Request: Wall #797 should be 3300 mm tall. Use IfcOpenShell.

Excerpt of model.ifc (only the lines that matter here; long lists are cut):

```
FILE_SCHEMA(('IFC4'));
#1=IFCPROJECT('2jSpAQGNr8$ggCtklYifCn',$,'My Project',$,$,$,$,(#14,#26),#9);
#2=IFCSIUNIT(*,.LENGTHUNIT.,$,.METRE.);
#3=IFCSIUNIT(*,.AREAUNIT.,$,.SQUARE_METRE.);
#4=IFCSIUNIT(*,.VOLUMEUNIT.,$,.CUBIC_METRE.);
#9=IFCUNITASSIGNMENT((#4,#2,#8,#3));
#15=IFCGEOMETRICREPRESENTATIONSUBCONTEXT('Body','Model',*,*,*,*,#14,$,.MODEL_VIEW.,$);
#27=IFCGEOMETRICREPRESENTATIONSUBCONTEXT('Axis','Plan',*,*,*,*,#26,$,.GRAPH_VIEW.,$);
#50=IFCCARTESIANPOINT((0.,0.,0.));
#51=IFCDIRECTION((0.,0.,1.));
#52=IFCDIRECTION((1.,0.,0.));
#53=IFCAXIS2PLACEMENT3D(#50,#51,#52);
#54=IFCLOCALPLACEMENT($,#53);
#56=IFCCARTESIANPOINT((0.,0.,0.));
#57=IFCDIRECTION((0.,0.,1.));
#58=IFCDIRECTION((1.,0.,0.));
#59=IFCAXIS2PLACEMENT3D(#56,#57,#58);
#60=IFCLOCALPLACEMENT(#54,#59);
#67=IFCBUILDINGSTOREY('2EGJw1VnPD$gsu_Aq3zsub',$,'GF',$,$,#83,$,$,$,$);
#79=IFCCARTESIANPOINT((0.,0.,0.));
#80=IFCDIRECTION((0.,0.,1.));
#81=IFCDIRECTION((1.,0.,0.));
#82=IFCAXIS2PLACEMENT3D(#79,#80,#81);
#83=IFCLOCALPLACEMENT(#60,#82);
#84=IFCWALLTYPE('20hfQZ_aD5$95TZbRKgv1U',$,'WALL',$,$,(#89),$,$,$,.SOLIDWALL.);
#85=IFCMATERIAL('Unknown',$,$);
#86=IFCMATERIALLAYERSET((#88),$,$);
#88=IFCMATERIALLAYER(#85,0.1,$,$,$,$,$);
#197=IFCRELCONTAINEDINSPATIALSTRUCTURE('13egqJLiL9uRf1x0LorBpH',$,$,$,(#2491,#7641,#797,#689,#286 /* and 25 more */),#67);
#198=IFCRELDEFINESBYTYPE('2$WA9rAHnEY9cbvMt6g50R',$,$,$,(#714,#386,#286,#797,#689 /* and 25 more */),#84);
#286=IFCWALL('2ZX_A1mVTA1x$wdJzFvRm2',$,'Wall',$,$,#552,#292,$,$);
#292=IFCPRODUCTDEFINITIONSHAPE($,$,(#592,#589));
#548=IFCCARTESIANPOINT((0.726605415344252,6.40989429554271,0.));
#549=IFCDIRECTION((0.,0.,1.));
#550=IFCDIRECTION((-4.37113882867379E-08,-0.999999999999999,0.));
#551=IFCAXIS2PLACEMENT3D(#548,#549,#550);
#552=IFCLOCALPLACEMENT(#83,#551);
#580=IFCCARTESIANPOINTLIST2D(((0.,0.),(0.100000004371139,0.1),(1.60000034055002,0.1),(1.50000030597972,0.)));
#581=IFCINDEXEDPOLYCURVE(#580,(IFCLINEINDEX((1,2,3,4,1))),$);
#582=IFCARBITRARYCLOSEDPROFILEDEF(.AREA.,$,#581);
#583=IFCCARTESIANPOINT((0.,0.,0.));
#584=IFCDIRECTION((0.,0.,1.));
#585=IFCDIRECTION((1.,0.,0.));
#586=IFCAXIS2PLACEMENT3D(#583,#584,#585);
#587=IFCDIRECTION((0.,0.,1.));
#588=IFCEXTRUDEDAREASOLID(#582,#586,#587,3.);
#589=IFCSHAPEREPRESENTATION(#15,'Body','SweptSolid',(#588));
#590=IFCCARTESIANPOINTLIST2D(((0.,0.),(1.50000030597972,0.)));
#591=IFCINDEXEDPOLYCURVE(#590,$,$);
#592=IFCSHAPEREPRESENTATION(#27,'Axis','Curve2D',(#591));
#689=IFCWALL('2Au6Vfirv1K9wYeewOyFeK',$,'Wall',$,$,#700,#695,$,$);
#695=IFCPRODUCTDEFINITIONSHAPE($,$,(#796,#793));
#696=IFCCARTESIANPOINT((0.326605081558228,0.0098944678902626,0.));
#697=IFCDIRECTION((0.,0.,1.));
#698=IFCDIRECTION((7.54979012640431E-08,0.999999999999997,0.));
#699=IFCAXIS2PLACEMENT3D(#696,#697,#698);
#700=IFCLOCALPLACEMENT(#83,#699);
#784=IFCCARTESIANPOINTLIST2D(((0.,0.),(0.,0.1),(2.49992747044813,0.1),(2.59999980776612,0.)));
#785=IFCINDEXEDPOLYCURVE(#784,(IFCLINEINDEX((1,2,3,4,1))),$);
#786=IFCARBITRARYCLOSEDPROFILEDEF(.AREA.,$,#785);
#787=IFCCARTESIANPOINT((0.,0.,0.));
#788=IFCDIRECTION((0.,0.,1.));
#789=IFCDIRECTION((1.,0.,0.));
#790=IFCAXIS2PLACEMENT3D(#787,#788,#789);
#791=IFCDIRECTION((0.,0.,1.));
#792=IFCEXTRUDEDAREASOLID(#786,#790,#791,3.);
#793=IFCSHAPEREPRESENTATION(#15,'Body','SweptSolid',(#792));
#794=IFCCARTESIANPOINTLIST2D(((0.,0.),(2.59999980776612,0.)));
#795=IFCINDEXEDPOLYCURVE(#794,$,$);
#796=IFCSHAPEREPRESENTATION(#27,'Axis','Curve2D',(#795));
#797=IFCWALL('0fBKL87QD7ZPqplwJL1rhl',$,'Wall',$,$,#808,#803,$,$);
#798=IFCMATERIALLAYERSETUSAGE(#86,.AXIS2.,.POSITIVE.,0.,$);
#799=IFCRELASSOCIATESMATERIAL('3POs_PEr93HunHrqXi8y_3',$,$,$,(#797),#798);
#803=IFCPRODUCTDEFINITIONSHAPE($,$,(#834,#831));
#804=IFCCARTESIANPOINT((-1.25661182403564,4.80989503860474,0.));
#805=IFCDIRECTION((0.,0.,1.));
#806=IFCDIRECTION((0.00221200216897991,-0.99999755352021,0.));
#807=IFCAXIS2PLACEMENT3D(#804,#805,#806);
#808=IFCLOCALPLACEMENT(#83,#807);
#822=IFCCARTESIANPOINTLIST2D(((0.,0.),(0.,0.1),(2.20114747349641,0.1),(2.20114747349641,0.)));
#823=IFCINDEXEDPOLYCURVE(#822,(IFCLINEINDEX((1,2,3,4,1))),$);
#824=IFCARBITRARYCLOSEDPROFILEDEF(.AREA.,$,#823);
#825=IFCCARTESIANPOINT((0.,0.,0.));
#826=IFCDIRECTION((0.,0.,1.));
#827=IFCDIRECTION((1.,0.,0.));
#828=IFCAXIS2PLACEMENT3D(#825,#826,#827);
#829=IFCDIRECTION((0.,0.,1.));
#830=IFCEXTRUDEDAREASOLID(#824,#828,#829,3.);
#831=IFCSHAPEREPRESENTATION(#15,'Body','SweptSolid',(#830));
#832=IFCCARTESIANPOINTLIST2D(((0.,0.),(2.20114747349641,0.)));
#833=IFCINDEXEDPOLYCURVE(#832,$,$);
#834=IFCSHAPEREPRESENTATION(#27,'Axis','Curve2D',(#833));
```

```python
import ifcopenshell
import ifcopenshell.geom
import ifcopenshell.util.representation
import ifcopenshell.util.shape
import ifcopenshell.util.unit

model = ifcopenshell.open("model.ifc")
unit_scale = ifcopenshell.util.unit.calculate_unit_scale(model)
settings = ifcopenshell.geom.settings()


def volume(element):
    """Net volume in cubic metres, openings subtracted."""
    shape = ifcopenshell.geom.create_shape(settings, element)
    return ifcopenshell.util.shape.get_volume(shape.geometry)


wall = model.by_id(797)
before = volume(wall)

body = ifcopenshell.util.representation.get_representation(wall, "Model", "Body")
solid = body.Items[0]
old_height = solid.Depth
solid.Depth = 3.3 / unit_scale
after = volume(wall)

print(f"height {old_height:g} -> {solid.Depth:g}, volume {before:.3f} -> {after:.3f} m3")

model.write("model-out.ifc")
```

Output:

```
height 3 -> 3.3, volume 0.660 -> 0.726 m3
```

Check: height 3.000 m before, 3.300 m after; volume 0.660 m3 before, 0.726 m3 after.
